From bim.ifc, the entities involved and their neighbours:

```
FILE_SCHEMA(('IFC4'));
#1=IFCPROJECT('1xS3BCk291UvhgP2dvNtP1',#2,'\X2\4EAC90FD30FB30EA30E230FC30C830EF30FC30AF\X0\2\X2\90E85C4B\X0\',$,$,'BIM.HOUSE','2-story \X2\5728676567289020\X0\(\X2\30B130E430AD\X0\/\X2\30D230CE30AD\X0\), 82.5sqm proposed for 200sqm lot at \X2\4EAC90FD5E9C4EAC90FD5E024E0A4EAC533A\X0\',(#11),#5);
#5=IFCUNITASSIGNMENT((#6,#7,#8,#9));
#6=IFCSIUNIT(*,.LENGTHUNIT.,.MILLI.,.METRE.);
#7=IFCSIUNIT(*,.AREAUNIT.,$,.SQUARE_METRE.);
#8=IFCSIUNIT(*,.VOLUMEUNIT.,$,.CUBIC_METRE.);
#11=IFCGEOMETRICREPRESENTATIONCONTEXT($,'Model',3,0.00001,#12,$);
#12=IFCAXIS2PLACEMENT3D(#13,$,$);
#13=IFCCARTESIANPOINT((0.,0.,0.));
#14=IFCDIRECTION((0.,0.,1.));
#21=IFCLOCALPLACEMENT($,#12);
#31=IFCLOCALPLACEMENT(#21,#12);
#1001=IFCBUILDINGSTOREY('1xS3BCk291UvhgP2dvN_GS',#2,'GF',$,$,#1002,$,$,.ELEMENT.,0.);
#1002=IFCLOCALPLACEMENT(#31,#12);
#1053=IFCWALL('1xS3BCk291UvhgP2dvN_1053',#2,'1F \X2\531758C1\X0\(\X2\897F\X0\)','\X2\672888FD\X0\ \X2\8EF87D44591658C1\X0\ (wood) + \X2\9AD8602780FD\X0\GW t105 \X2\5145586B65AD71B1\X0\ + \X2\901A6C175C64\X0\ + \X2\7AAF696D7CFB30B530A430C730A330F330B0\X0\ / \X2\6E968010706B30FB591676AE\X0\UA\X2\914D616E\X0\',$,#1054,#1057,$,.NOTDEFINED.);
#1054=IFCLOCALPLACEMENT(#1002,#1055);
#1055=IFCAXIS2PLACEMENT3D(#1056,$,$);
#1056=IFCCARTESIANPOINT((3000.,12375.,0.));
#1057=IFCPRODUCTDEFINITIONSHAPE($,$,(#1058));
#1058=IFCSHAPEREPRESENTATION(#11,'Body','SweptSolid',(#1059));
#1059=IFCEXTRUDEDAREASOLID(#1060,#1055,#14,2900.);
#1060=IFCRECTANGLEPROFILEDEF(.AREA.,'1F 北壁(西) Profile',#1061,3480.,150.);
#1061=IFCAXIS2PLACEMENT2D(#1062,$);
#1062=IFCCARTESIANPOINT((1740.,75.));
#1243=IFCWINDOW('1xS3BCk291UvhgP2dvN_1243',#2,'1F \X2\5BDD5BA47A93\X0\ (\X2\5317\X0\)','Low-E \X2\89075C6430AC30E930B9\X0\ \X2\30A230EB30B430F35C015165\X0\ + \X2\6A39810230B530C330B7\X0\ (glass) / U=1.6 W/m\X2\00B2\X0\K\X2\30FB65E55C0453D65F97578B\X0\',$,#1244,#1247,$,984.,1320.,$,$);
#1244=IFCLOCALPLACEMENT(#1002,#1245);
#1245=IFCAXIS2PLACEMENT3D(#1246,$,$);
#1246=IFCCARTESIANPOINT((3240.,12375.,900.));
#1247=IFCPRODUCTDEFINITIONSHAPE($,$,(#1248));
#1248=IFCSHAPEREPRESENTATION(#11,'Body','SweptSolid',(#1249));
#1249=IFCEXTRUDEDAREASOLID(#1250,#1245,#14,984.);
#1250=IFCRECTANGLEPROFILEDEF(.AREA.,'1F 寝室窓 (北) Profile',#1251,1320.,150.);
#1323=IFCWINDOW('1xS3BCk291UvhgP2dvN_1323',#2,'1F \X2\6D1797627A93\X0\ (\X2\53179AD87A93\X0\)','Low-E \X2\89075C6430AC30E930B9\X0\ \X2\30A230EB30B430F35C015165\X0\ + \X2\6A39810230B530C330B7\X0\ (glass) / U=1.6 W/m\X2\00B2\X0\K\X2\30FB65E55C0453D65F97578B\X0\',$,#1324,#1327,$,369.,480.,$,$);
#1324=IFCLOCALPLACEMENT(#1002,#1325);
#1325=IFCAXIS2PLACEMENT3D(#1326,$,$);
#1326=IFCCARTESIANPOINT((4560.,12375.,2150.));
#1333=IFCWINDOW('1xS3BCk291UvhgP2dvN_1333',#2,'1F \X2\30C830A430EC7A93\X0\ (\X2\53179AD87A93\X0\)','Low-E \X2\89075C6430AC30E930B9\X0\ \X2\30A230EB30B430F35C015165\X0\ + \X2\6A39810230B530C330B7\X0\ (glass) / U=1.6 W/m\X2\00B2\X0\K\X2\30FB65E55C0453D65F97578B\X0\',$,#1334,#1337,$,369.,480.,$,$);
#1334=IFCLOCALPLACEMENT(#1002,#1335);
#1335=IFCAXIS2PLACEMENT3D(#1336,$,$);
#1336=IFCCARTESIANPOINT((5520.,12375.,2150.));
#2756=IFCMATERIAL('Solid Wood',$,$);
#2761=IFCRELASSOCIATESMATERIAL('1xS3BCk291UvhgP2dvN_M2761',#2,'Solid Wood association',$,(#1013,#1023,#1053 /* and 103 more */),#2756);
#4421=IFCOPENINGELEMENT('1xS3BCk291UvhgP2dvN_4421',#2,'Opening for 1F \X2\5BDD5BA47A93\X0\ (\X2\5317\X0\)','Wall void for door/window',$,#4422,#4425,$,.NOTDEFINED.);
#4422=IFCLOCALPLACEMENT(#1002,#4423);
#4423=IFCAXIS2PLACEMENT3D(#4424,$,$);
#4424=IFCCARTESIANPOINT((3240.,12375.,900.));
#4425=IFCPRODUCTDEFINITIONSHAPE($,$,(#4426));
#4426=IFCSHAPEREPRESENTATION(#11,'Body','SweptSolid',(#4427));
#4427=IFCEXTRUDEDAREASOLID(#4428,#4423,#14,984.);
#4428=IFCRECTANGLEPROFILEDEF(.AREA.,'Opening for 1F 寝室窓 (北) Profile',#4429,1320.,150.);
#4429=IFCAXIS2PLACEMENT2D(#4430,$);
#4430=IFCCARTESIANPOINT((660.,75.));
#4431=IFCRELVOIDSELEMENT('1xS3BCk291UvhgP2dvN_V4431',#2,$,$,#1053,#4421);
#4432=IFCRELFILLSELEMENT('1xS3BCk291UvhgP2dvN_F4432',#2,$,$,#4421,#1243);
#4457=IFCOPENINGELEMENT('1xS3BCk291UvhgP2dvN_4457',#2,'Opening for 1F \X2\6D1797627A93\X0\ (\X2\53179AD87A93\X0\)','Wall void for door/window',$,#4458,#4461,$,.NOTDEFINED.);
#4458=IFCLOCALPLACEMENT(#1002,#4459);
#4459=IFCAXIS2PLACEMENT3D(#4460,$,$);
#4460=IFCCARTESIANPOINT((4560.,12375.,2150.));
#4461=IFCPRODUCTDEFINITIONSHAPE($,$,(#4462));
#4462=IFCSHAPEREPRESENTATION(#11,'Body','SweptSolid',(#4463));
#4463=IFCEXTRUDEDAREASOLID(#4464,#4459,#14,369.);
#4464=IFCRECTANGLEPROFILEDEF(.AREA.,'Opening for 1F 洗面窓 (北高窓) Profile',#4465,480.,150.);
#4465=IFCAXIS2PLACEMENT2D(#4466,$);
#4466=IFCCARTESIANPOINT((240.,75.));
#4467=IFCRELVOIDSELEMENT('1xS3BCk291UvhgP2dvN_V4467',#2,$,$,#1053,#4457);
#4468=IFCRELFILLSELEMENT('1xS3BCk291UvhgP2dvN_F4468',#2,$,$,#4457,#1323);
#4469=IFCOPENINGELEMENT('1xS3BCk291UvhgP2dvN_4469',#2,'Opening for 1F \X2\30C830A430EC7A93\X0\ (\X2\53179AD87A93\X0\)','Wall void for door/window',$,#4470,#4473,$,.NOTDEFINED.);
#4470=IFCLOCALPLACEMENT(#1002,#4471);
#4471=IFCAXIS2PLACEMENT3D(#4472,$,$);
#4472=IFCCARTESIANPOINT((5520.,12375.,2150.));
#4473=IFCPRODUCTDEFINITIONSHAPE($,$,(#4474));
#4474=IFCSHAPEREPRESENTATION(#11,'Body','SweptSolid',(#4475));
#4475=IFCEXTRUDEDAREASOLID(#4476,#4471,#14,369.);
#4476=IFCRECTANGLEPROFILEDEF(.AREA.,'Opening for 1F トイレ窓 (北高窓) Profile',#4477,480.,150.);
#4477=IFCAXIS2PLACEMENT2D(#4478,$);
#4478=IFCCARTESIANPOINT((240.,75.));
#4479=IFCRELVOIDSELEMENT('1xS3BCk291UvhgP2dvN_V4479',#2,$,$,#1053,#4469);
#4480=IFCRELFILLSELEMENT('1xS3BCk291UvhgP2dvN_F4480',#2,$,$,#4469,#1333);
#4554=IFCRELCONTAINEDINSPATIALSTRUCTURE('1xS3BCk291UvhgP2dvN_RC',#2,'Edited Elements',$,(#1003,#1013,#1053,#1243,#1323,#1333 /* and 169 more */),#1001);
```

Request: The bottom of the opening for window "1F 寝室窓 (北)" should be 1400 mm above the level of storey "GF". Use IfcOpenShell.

```python
import numpy as np
import ifcopenshell
import ifcopenshell.api.geometry
import ifcopenshell.geom
import ifcopenshell.util.element
import ifcopenshell.util.placement
import ifcopenshell.util.shape
import ifcopenshell.util.unit

model = ifcopenshell.open("bim.ifc")
unit_scale = ifcopenshell.util.unit.calculate_unit_scale(model)

window = model.by_id(1243)
opening = window.FillsVoids[0].RelatingOpeningElement
storey = ifcopenshell.util.element.get_container(window, ifc_class="IfcBuildingStorey")
level = ifcopenshell.util.placement.get_local_placement(storey.ObjectPlacement)[2, 3]

# The opening's origin need not be at the sill, so measure its lowest point.
shape = ifcopenshell.geom.create_shape(ifcopenshell.geom.settings(), opening)
bottom = ifcopenshell.util.shape.get_shape_bottom_elevation(shape, shape.geometry) / unit_scale
dz = level + 1.4 / unit_scale - bottom

shift = np.array([0.0, 0.0, dz])
# The window is not placed relative to its opening, so move both.
for product in (opening, window):
    matrix = ifcopenshell.util.placement.get_local_placement(product.ObjectPlacement)
    matrix[:3, 3] += shift
    ifcopenshell.api.geometry.edit_object_placement(model, product=product, matrix=matrix, is_si=False)

print(f"moved by {dz * unit_scale:+.3f} m")

model.write("bim_updated.ifc")
```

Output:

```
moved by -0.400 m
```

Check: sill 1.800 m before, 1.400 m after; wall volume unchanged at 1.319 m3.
